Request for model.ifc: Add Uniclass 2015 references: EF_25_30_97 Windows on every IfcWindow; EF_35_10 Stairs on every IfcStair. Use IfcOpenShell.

First a look at what the model holds.

```python
import ifcopenshell

model = ifcopenshell.open("model.ifc")
print(model.schema)
print("classifications:", [c.Name for c in model.by_type("IfcClassification")])
for ifc_class in ("IfcDoor", "IfcRoof", "IfcStair", "IfcWall", "IfcWindow"):
    print(ifc_class, len(model.by_type(ifc_class)))
```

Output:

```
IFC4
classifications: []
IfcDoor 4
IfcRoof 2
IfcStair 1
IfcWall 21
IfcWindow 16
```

```python
import ifcopenshell
import ifcopenshell.api.classification

model = ifcopenshell.open("model.ifc")

system = ifcopenshell.api.classification.add_classification(model, classification="Uniclass 2015")

codes = {
    "IfcWindow": ("EF_25_30_97", "Windows"),
    "IfcStair": ("EF_35_10", "Stairs"),
}
for ifc_class, (code, name) in codes.items():
    products = model.by_type(ifc_class)
    ifcopenshell.api.classification.add_reference(
        model, products=products, classification=system, identification=code, name=name
    )
    print(code, len(products))

model.write("model_updated.ifc")
```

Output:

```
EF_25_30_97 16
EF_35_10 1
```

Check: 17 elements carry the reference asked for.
